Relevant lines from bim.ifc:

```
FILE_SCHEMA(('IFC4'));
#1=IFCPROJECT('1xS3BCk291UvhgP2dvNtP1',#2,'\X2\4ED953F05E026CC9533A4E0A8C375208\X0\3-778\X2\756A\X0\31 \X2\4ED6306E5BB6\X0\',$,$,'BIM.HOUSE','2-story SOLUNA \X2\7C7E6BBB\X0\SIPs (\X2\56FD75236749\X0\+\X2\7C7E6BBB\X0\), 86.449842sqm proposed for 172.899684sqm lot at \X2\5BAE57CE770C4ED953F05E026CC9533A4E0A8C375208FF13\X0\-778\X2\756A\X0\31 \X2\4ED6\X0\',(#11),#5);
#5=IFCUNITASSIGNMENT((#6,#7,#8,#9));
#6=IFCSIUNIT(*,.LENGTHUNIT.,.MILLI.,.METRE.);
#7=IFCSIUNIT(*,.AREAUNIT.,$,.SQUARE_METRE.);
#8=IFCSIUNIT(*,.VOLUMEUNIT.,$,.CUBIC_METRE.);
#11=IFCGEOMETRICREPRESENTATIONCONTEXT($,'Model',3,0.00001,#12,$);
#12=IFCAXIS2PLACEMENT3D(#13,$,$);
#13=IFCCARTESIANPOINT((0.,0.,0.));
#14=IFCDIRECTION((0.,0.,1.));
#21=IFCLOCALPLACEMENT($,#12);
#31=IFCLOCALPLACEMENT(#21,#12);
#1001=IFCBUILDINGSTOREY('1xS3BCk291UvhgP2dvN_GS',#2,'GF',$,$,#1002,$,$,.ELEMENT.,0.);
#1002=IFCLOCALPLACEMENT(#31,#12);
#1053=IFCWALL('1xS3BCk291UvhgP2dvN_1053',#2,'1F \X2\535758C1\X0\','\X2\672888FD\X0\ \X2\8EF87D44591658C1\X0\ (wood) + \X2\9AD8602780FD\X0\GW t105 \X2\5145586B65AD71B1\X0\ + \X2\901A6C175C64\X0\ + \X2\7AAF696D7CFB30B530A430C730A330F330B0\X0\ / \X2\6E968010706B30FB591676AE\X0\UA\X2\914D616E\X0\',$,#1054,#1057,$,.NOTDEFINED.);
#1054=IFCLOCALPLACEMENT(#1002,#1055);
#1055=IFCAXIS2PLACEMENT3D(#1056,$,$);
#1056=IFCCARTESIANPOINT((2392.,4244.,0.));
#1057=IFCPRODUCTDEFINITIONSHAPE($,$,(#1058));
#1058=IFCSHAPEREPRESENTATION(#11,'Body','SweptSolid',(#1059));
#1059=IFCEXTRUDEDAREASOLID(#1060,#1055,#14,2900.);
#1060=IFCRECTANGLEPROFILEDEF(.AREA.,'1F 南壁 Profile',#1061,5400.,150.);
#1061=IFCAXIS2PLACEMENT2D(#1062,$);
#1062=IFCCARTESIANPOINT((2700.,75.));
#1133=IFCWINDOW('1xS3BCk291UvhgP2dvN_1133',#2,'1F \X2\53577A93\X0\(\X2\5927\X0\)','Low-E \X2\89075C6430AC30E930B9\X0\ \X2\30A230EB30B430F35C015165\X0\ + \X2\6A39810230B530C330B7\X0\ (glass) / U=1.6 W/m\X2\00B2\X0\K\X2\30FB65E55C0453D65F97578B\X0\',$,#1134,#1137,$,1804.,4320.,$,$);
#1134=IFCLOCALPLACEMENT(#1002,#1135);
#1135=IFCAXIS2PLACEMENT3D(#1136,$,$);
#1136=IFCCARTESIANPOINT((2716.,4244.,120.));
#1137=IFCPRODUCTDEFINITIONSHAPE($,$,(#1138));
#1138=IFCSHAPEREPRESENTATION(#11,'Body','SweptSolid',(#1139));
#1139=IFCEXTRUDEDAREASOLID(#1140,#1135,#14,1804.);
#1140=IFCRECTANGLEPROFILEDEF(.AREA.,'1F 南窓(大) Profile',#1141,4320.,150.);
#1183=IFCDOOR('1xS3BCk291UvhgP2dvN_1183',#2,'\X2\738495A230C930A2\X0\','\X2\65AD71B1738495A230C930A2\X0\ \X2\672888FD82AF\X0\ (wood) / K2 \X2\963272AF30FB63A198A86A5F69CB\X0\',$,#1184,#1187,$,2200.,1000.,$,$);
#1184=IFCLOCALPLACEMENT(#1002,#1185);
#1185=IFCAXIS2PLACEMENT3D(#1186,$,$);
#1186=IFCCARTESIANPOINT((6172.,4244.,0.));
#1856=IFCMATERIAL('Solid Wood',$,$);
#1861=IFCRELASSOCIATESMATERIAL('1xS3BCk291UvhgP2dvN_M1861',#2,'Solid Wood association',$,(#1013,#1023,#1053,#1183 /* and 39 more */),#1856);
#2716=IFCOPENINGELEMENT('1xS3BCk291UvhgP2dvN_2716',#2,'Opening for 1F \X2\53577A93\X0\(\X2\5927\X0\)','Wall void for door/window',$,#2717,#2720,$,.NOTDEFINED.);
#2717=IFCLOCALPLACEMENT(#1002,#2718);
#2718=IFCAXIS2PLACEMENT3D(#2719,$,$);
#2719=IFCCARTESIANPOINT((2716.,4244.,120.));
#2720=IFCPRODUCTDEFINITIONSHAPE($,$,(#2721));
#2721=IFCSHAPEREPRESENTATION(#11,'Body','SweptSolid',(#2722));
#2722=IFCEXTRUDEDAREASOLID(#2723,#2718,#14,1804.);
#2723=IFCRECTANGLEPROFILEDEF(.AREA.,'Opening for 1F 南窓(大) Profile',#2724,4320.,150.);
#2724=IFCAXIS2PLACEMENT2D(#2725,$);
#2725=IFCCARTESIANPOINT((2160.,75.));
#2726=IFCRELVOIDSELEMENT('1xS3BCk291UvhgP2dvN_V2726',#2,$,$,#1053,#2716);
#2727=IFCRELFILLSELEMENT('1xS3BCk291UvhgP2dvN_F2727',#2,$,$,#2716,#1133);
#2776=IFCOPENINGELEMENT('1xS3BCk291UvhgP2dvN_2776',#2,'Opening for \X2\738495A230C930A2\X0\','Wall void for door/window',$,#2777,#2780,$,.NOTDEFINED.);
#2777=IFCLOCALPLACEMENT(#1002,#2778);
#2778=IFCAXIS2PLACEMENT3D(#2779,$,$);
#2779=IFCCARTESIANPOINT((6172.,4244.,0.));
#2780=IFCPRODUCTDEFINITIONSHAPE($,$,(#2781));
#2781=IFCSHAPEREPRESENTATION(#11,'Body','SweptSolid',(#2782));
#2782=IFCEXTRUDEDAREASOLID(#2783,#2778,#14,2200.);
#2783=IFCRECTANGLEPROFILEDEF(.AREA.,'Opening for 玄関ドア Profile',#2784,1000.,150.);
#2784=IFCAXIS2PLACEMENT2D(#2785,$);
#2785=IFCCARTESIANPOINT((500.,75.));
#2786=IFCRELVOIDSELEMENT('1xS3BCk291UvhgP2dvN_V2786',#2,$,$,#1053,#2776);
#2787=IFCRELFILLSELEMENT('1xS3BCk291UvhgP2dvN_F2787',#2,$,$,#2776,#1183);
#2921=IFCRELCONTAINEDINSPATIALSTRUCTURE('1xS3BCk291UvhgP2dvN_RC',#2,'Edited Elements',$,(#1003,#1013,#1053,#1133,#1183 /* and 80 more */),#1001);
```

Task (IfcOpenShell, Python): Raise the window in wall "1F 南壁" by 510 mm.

```python
import numpy as np
import ifcopenshell
import ifcopenshell.api.geometry
import ifcopenshell.util.placement
import ifcopenshell.util.unit

model = ifcopenshell.open("bim.ifc")
unit_scale = ifcopenshell.util.unit.calculate_unit_scale(model)

window = model.by_id(1133)
opening = window.FillsVoids[0].RelatingOpeningElement
dz = 0.51 / unit_scale

shift = np.array([0.0, 0.0, dz])
# The window is not placed relative to its opening, so move both.
for product in (opening, window):
    matrix = ifcopenshell.util.placement.get_local_placement(product.ObjectPlacement)
    matrix[:3, 3] += shift
    ifcopenshell.api.geometry.edit_object_placement(model, product=product, matrix=matrix, is_si=False)

print(f"moved by {dz * unit_scale:+.3f} m")

model.write("bim-out.ifc")
```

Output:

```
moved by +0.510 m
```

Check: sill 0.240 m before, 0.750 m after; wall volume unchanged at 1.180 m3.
